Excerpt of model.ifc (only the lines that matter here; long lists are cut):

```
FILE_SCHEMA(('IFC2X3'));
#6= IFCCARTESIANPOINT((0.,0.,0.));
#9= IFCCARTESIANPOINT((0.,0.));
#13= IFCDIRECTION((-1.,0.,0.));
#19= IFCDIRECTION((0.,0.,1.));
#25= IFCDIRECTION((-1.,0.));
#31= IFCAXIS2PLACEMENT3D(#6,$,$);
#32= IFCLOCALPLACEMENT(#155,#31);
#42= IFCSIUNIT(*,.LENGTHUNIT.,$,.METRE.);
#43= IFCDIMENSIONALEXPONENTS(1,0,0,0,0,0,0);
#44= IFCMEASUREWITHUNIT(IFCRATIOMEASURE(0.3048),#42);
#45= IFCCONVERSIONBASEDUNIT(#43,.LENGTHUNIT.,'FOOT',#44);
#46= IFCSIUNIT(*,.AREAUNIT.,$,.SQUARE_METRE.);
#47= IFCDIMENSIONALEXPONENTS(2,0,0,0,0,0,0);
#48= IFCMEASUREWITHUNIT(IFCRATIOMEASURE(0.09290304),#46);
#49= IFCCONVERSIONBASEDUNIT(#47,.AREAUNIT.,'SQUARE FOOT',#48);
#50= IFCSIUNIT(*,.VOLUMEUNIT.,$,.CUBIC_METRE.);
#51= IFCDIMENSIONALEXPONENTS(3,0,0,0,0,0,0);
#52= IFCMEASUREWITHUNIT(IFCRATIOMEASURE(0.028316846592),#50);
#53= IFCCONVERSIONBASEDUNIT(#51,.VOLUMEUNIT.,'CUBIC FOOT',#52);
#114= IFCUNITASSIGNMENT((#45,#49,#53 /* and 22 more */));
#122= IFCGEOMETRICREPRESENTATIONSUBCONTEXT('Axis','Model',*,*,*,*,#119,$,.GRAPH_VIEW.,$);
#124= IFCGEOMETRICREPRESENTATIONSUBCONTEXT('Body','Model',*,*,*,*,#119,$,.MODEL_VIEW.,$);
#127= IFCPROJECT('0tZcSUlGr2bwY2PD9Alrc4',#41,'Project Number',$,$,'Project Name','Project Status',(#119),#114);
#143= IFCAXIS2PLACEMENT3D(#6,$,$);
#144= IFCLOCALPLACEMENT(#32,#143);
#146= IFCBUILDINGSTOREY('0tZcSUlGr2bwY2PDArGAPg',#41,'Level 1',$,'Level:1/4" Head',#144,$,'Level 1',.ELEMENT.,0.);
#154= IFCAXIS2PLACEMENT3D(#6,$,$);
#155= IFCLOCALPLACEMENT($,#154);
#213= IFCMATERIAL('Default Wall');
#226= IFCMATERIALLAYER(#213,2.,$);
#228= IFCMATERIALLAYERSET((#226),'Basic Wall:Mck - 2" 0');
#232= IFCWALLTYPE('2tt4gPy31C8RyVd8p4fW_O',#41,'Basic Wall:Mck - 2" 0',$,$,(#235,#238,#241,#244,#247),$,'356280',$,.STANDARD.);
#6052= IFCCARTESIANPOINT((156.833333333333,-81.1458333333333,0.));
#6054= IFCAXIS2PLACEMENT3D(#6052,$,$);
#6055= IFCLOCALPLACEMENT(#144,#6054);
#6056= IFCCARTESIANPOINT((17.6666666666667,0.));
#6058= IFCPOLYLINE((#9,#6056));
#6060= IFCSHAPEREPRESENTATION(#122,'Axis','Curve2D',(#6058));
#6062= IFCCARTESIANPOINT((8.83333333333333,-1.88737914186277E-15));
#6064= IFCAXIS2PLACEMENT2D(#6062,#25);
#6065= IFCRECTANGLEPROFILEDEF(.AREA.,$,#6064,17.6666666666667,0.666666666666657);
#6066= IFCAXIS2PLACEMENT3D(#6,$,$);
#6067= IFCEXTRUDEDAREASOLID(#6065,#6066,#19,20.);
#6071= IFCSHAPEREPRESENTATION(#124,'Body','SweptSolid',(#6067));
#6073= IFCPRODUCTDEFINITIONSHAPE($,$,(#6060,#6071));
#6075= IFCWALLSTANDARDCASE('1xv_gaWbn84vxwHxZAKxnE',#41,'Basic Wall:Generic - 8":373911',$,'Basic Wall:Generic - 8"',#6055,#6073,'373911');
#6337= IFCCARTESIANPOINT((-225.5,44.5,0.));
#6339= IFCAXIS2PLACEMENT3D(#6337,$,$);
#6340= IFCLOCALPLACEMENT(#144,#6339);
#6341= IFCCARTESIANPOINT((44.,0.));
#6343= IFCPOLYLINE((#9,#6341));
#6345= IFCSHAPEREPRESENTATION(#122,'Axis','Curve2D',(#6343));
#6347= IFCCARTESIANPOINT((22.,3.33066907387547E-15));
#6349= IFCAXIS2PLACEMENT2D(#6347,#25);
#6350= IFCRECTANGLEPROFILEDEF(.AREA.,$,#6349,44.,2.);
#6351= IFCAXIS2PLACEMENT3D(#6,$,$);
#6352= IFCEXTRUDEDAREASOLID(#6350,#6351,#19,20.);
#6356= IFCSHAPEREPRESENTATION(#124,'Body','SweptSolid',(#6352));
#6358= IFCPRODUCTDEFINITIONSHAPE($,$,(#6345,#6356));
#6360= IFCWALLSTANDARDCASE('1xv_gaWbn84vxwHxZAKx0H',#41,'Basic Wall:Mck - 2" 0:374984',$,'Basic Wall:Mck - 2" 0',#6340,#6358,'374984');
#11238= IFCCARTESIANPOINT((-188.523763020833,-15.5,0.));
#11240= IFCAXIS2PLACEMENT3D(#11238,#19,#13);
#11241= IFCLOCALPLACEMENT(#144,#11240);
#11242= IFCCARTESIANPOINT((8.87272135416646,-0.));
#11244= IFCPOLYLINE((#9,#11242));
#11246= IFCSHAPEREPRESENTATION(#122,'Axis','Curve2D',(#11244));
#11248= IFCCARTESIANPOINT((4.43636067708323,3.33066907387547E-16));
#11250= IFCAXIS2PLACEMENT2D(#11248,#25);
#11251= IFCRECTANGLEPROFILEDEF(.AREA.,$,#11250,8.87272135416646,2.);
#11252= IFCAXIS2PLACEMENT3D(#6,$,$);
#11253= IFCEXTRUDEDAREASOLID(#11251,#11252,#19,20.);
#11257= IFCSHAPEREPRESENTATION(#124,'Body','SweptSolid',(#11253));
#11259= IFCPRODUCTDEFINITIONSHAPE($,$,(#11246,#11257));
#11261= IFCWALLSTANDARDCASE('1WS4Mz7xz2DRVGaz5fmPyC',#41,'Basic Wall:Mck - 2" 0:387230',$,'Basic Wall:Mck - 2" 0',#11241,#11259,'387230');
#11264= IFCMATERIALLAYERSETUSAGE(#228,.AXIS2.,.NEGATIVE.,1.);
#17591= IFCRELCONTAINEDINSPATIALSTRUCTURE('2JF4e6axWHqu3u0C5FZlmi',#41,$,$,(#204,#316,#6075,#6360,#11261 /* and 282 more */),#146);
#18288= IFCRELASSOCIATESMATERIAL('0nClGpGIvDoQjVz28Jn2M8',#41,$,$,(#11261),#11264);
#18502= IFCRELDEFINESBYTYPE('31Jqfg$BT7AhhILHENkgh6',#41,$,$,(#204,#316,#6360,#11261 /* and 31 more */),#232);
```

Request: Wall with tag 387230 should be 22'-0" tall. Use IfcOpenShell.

```python
import ifcopenshell
import ifcopenshell.geom
import ifcopenshell.util.representation
import ifcopenshell.util.shape
import ifcopenshell.util.unit

model = ifcopenshell.open("model.ifc")
unit_scale = ifcopenshell.util.unit.calculate_unit_scale(model)
settings = ifcopenshell.geom.settings()


def volume(element):
    """Net volume in cubic metres, openings subtracted."""
    shape = ifcopenshell.geom.create_shape(settings, element)
    return ifcopenshell.util.shape.get_volume(shape.geometry)


wall = model.by_guid("1WS4Mz7xz2DRVGaz5fmPyC")
before = volume(wall)

body = ifcopenshell.util.representation.get_representation(wall, "Model", "Body")
solid = body.Items[0]
old_height = solid.Depth
solid.Depth = 264 * 0.0254 / unit_scale
after = volume(wall)

print(f"height {old_height:g} -> {solid.Depth:g}, volume {before:.3f} -> {after:.3f} m3")

model.write("model-out.ifc")
```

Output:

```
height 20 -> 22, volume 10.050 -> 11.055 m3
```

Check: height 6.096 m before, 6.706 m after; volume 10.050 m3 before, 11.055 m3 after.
